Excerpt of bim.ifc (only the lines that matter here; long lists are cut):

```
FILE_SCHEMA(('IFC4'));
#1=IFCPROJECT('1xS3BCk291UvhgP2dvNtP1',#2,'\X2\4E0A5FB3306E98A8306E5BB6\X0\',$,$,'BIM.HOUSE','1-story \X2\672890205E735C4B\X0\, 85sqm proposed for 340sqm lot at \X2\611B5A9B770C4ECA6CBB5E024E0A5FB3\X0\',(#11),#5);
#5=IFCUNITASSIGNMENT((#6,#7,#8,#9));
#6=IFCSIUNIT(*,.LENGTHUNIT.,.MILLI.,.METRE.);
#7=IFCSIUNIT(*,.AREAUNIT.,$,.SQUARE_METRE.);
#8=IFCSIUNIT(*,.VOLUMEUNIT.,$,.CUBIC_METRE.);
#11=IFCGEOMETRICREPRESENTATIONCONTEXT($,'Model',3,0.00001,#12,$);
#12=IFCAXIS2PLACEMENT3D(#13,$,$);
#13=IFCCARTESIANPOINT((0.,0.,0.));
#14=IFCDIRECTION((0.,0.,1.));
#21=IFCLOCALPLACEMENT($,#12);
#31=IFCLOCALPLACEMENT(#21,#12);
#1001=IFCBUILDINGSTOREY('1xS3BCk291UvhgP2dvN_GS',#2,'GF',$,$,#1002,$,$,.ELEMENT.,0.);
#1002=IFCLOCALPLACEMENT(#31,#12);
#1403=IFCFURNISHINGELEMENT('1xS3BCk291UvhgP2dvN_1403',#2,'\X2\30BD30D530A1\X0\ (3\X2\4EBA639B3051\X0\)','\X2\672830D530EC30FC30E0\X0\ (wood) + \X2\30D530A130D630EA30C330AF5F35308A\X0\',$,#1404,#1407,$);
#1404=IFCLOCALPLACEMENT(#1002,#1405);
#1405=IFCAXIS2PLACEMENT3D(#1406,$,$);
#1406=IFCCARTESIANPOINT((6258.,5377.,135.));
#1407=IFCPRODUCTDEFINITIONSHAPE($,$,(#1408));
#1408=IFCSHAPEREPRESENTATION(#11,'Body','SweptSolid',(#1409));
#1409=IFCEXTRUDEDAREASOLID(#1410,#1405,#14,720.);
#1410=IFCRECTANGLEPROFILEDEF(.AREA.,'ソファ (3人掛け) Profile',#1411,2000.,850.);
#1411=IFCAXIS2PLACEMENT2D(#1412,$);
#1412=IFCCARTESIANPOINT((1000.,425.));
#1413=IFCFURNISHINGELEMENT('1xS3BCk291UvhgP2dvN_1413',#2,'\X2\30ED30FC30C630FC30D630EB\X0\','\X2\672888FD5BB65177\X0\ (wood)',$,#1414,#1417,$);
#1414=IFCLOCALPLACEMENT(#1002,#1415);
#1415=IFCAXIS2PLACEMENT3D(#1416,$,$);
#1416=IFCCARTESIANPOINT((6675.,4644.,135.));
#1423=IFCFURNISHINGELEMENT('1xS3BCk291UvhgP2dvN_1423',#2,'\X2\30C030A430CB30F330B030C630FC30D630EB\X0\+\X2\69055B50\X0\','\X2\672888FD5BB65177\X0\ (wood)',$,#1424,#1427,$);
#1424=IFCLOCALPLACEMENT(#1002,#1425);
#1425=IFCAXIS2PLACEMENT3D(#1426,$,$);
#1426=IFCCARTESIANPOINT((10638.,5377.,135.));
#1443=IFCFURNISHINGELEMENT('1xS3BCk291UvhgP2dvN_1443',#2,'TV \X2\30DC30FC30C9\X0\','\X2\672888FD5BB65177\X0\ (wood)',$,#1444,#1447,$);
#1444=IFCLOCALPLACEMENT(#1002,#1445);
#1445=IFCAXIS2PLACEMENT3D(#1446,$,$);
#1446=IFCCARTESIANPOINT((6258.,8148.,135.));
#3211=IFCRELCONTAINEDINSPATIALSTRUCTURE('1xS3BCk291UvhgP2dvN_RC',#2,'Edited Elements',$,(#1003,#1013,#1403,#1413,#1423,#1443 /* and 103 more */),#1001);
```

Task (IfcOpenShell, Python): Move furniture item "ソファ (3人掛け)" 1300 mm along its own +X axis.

```python
import ifcopenshell
import ifcopenshell.api.geometry
import ifcopenshell.util.placement
import ifcopenshell.util.unit

model = ifcopenshell.open("bim.ifc")
unit_scale = ifcopenshell.util.unit.calculate_unit_scale(model)

item = model.by_guid("1xS3BCk291UvhgP2dvN_1403")
matrix = ifcopenshell.util.placement.get_local_placement(item.ObjectPlacement)
matrix[:3, 3] += matrix[:3, 0] * 1.3 / unit_scale
ifcopenshell.api.geometry.edit_object_placement(model, product=item, matrix=matrix, is_si=False)

print(ifcopenshell.util.placement.get_local_placement(item.ObjectPlacement).round(3) + 0.0)

model.write("bim_rev.ifc")
```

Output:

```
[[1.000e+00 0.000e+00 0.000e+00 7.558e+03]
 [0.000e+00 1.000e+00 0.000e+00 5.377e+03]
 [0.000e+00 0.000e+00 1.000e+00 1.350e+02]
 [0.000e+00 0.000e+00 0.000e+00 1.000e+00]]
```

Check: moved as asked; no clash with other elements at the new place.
